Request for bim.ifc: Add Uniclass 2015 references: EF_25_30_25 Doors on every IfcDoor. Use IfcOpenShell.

First a look at what the model holds.

```python
import ifcopenshell

model = ifcopenshell.open("bim.ifc")
print(model.schema)
print("classifications:", [c.Name for c in model.by_type("IfcClassification")])
for ifc_class in ("IfcDoor", "IfcRoof", "IfcStair", "IfcWall", "IfcWindow"):
    print(ifc_class, len(model.by_type(ifc_class)))
```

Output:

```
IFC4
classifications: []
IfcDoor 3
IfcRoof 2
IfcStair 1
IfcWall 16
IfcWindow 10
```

```python
import ifcopenshell
import ifcopenshell.api.classification

model = ifcopenshell.open("bim.ifc")

system = ifcopenshell.api.classification.add_classification(model, classification="Uniclass 2015")

codes = {
    "IfcDoor": ("EF_25_30_25", "Doors"),
}
for ifc_class, (code, name) in codes.items():
    products = model.by_type(ifc_class)
    ifcopenshell.api.classification.add_reference(
        model, products=products, classification=system, identification=code, name=name
    )
    print(code, len(products))

model.write("bim_rev.ifc")
```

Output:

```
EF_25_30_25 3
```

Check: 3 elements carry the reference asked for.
